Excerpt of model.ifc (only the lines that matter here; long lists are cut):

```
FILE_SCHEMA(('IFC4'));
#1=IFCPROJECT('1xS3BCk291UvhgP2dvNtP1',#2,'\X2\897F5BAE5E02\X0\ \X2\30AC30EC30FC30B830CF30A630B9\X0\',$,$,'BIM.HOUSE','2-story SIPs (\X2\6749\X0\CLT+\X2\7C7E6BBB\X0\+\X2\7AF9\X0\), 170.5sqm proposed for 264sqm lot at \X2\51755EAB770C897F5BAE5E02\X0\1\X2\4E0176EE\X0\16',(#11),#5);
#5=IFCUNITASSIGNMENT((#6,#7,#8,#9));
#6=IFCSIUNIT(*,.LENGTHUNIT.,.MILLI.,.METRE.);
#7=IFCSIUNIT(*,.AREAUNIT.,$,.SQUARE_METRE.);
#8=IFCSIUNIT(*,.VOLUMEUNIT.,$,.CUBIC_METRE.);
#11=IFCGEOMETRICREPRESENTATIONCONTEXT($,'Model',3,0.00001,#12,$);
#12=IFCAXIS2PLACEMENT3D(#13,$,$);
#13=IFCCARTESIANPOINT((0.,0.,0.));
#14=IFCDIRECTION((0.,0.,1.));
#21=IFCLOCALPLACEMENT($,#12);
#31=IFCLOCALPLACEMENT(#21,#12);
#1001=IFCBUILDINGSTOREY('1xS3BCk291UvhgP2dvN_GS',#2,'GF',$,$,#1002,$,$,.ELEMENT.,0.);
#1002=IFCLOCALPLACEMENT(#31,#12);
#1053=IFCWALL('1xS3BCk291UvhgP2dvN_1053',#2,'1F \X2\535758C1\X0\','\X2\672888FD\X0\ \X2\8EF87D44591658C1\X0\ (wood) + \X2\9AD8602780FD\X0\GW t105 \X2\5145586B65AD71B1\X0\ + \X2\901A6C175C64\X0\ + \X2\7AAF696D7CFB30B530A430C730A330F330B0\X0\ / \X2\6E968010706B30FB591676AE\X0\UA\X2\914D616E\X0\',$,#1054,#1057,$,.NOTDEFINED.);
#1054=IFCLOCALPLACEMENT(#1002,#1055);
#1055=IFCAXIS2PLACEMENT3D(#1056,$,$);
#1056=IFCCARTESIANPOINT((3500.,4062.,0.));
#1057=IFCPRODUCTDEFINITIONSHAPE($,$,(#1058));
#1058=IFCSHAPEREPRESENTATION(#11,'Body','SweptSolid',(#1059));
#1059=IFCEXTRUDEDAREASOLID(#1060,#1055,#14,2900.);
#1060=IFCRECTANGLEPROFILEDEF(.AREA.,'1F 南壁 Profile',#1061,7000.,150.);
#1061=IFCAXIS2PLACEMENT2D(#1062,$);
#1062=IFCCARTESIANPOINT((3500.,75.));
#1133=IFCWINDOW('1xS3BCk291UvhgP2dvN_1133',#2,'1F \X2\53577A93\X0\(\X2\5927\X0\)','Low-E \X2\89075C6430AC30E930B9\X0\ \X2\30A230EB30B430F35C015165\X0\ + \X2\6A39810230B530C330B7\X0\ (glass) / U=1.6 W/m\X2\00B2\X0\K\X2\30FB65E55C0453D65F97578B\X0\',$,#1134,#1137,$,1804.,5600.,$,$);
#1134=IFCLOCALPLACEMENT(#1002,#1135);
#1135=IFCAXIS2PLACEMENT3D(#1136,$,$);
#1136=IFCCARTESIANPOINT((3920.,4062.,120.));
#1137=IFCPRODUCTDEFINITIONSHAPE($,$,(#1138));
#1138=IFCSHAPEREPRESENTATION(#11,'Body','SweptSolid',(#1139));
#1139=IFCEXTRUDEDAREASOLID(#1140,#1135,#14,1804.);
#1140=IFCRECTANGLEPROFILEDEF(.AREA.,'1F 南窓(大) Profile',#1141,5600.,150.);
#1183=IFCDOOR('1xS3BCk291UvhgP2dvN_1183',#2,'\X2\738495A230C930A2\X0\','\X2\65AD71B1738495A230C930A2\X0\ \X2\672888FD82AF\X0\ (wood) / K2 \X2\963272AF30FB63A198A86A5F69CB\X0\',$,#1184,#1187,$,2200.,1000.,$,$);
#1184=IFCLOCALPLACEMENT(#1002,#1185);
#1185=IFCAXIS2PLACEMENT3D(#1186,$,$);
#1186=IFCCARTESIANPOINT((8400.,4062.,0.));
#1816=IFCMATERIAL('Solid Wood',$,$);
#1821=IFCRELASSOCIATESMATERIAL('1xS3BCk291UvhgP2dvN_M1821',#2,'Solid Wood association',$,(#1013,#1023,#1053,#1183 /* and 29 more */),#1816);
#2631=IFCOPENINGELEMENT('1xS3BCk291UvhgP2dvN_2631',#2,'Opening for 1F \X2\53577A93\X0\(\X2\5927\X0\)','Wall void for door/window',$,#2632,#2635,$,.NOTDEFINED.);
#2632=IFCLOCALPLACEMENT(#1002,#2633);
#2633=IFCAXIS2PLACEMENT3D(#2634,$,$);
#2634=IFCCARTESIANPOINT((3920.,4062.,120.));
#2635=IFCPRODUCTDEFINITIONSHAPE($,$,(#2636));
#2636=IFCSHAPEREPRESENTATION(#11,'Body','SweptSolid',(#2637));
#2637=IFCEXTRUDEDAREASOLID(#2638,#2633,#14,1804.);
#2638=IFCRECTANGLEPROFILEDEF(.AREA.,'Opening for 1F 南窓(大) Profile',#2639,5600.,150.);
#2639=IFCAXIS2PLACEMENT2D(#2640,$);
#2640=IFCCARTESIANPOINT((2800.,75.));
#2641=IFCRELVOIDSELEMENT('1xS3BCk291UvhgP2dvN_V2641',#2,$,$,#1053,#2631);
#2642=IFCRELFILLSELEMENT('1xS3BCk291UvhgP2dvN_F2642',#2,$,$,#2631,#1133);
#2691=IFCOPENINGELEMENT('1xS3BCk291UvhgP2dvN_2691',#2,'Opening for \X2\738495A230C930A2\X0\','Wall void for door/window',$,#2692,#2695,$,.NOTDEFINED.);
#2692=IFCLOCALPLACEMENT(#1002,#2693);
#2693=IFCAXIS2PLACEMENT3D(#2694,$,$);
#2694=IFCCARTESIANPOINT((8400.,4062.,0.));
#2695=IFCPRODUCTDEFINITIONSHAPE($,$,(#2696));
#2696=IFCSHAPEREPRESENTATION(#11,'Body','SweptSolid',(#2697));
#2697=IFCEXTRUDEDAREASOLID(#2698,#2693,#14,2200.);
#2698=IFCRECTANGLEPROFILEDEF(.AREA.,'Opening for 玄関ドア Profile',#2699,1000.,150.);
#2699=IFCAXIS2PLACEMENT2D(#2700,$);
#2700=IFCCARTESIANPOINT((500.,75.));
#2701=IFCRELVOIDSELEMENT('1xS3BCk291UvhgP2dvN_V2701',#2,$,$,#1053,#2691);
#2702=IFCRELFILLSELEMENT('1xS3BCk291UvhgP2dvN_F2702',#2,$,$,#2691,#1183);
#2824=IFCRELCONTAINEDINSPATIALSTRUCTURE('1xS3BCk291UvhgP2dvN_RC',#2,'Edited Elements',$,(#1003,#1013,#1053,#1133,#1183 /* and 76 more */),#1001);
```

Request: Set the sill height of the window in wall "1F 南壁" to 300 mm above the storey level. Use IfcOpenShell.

```python
import numpy as np
import ifcopenshell
import ifcopenshell.api.geometry
import ifcopenshell.geom
import ifcopenshell.util.element
import ifcopenshell.util.placement
import ifcopenshell.util.shape
import ifcopenshell.util.unit

model = ifcopenshell.open("model.ifc")
unit_scale = ifcopenshell.util.unit.calculate_unit_scale(model)

window = model.by_guid("1xS3BCk291UvhgP2dvN_1133")
opening = window.FillsVoids[0].RelatingOpeningElement
storey = ifcopenshell.util.element.get_container(window, ifc_class="IfcBuildingStorey")
level = ifcopenshell.util.placement.get_local_placement(storey.ObjectPlacement)[2, 3]

# The opening's origin need not be at the sill, so measure its lowest point.
shape = ifcopenshell.geom.create_shape(ifcopenshell.geom.settings(), opening)
bottom = ifcopenshell.util.shape.get_shape_bottom_elevation(shape, shape.geometry) / unit_scale
dz = level + 0.3 / unit_scale - bottom

shift = np.array([0.0, 0.0, dz])
# The window is not placed relative to its opening, so move both.
for product in (opening, window):
    matrix = ifcopenshell.util.placement.get_local_placement(product.ObjectPlacement)
    matrix[:3, 3] += shift
    ifcopenshell.api.geometry.edit_object_placement(model, product=product, matrix=matrix, is_si=False)

print(f"moved by {dz * unit_scale:+.3f} m")

model.write("model_v2.ifc")
```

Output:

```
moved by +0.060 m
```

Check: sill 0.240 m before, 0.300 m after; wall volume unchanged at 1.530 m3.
